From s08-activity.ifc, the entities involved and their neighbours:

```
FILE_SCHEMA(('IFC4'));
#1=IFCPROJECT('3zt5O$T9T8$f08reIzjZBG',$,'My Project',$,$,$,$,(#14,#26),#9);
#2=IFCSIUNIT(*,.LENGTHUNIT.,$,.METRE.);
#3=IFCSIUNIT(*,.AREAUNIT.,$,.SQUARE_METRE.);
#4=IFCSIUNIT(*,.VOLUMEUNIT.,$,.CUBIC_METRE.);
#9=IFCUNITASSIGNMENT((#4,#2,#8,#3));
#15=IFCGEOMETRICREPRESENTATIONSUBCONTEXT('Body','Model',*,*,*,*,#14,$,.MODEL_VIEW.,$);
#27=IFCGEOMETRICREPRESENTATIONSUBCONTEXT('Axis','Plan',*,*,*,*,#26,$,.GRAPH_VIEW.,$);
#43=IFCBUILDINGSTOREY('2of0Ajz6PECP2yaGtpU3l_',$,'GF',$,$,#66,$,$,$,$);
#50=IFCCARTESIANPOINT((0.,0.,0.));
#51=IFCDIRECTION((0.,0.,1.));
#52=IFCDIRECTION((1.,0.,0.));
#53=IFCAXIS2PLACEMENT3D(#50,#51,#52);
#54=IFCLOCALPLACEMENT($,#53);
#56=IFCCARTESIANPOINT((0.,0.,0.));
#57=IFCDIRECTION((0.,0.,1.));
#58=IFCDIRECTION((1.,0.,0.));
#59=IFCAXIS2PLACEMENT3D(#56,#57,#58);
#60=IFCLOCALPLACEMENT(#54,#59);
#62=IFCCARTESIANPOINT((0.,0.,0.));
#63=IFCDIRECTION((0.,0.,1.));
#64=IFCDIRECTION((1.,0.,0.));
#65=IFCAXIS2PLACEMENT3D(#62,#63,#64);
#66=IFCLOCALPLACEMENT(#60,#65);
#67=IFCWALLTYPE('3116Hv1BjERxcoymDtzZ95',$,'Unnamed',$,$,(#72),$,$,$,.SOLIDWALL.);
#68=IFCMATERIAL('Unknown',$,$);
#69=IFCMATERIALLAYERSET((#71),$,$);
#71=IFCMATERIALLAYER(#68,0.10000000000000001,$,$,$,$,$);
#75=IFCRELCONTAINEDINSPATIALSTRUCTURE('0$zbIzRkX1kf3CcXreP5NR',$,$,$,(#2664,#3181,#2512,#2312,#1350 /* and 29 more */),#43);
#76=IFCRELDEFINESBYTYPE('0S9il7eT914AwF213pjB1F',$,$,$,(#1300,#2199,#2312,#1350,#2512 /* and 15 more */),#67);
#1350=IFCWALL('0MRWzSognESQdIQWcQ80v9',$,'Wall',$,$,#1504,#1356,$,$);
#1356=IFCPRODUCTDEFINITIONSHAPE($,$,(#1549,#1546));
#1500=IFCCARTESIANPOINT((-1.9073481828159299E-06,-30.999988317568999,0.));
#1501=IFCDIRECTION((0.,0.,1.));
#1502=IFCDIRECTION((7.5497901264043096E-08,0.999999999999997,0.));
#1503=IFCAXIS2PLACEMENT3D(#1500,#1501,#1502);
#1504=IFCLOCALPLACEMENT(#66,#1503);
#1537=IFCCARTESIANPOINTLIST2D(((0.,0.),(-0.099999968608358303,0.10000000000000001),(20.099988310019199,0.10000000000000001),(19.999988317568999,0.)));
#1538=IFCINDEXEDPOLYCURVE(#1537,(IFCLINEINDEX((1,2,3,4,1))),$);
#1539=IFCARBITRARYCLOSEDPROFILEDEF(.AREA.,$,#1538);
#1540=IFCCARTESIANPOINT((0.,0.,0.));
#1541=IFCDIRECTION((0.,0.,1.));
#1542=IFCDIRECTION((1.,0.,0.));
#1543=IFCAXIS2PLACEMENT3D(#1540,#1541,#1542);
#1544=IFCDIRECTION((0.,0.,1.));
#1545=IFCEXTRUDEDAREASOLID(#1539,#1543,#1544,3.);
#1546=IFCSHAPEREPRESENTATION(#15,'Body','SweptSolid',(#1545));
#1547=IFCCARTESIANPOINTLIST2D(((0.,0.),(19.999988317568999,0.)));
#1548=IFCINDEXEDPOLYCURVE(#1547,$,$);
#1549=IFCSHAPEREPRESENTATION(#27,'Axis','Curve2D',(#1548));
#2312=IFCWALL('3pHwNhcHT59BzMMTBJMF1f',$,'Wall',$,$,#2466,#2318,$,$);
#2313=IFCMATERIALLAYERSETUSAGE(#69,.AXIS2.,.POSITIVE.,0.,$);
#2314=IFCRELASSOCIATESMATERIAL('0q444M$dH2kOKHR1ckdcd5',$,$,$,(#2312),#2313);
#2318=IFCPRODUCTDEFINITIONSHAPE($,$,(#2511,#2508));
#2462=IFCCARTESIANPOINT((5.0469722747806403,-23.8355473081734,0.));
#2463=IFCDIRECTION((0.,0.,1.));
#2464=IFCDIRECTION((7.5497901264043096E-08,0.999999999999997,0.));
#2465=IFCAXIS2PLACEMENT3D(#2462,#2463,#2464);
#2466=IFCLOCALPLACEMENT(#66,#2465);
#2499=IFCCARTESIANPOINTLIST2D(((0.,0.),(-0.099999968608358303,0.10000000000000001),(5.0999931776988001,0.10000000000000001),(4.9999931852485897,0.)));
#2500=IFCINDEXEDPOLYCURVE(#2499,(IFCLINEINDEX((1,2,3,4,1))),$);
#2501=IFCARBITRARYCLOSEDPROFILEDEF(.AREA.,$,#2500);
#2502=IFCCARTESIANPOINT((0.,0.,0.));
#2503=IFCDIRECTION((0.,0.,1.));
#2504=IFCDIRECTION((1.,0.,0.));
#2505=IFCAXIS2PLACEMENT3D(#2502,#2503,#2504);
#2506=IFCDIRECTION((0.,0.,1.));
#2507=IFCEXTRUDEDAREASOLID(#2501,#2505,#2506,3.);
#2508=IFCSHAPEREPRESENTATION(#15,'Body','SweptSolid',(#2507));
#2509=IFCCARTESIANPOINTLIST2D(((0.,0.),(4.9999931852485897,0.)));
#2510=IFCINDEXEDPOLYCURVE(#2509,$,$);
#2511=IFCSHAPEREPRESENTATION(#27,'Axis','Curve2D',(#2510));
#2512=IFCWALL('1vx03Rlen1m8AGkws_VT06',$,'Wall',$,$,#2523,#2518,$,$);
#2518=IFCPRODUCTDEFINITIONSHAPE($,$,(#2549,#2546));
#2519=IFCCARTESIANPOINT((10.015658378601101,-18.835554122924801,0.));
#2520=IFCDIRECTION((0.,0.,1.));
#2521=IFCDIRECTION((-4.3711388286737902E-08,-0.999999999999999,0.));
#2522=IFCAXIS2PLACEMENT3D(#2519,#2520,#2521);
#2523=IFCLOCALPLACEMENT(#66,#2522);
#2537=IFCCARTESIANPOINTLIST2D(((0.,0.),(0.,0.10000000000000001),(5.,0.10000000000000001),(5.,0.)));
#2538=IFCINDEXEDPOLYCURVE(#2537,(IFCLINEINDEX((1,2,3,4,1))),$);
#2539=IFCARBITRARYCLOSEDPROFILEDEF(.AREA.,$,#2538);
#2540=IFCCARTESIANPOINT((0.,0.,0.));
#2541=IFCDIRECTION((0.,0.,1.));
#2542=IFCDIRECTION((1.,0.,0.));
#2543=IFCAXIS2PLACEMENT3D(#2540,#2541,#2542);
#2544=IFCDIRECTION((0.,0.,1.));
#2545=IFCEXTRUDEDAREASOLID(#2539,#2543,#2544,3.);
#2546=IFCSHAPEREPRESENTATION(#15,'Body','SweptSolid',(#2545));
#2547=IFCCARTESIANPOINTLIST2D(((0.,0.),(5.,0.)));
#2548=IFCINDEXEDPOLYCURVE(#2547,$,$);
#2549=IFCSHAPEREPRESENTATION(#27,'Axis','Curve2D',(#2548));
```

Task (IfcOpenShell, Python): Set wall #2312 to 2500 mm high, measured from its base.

```python
import ifcopenshell
import ifcopenshell.geom
import ifcopenshell.util.representation
import ifcopenshell.util.shape
import ifcopenshell.util.unit

model = ifcopenshell.open("s08-activity.ifc")
unit_scale = ifcopenshell.util.unit.calculate_unit_scale(model)
settings = ifcopenshell.geom.settings()


def volume(element):
    """Net volume in cubic metres, openings subtracted."""
    shape = ifcopenshell.geom.create_shape(settings, element)
    return ifcopenshell.util.shape.get_volume(shape.geometry)


wall = model.by_guid("3pHwNhcHT59BzMMTBJMF1f")
before = volume(wall)

body = ifcopenshell.util.representation.get_representation(wall, "Model", "Body")
solid = body.Items[0]
old_height = solid.Depth
solid.Depth = 2.5 / unit_scale
after = volume(wall)

print(f"height {old_height:g} -> {solid.Depth:g}, volume {before:.3f} -> {after:.3f} m3")

model.write("s08-activity-out.ifc")
```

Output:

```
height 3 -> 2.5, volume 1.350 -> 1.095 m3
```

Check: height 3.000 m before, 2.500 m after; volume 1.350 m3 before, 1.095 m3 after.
